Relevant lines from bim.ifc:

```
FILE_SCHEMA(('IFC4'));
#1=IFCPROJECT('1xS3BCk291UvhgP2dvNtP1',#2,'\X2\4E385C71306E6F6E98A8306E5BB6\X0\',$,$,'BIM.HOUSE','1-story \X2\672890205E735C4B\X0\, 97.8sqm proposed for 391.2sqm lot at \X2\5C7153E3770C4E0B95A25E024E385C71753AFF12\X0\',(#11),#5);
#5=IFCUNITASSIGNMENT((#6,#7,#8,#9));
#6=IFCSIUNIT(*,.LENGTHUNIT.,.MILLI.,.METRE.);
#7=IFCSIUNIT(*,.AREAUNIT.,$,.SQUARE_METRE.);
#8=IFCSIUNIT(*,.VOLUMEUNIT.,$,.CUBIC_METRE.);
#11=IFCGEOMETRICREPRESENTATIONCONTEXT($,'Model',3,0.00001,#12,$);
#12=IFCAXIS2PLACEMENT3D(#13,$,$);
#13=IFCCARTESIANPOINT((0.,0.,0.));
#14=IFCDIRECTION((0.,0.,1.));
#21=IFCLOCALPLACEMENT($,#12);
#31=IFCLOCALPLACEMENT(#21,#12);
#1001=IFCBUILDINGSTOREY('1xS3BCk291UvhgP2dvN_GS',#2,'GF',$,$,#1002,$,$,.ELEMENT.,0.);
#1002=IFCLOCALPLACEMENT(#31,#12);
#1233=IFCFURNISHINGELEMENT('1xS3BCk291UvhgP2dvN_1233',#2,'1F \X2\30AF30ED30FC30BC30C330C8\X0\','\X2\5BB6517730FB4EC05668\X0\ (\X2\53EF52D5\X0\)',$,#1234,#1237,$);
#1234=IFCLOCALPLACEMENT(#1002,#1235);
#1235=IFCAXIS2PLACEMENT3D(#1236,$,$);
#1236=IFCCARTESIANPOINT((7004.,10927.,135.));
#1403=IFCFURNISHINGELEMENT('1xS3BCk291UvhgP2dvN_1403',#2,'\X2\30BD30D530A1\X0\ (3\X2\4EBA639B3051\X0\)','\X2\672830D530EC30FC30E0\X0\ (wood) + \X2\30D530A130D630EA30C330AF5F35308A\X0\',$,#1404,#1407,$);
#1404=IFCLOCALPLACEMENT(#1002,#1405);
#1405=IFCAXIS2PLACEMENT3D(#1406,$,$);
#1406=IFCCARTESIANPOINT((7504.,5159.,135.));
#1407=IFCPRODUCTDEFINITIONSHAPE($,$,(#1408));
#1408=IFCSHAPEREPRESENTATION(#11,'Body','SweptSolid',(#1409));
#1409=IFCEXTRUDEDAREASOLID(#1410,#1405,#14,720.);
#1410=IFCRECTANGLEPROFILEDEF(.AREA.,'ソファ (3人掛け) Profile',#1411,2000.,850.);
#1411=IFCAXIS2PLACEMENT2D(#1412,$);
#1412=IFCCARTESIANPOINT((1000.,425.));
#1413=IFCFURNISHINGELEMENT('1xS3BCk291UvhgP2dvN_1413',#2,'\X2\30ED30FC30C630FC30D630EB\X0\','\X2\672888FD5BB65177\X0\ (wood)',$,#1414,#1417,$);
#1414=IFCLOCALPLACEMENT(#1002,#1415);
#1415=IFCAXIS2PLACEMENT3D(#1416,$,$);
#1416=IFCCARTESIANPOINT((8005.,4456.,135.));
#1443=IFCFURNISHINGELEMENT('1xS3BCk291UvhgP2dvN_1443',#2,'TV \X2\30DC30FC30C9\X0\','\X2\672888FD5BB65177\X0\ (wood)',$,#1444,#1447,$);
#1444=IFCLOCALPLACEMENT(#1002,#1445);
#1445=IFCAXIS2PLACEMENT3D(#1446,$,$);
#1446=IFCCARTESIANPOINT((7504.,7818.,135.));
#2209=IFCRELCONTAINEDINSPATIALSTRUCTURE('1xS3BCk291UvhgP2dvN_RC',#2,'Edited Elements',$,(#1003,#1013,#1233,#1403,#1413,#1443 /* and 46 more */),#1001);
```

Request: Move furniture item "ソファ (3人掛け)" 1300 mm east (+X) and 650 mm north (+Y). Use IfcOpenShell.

```python
import ifcopenshell
import ifcopenshell.api.geometry
import ifcopenshell.util.placement
import ifcopenshell.util.unit

model = ifcopenshell.open("bim.ifc")
unit_scale = ifcopenshell.util.unit.calculate_unit_scale(model)

item = model.by_id(1403)
matrix = ifcopenshell.util.placement.get_local_placement(item.ObjectPlacement)
matrix[0, 3] += 1.3 / unit_scale
matrix[1, 3] += 0.65 / unit_scale
ifcopenshell.api.geometry.edit_object_placement(model, product=item, matrix=matrix, is_si=False)

print(ifcopenshell.util.placement.get_local_placement(item.ObjectPlacement).round(3) + 0.0)

model.write("bim_edited.ifc")
```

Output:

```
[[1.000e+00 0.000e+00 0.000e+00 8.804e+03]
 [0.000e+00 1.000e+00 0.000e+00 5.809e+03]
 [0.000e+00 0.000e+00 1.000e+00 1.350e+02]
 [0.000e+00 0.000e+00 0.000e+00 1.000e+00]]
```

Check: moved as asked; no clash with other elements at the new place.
